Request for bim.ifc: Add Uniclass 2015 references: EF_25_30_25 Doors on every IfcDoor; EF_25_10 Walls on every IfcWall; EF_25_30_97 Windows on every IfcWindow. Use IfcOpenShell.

First a look at what the model holds.

```python
import ifcopenshell

model = ifcopenshell.open("bim.ifc")
print(model.schema)
print("classifications:", [c.Name for c in model.by_type("IfcClassification")])
for ifc_class in ("IfcDoor", "IfcRoof", "IfcStair", "IfcWall", "IfcWindow"):
    print(ifc_class, len(model.by_type(ifc_class)))
```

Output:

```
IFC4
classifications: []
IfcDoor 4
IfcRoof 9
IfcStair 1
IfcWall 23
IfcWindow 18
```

```python
import ifcopenshell
import ifcopenshell.api.classification

model = ifcopenshell.open("bim.ifc")

system = ifcopenshell.api.classification.add_classification(model, classification="Uniclass 2015")

codes = {
    "IfcDoor": ("EF_25_30_25", "Doors"),
    "IfcWall": ("EF_25_10", "Walls"),
    "IfcWindow": ("EF_25_30_97", "Windows"),
}
for ifc_class, (code, name) in codes.items():
    products = model.by_type(ifc_class)
    ifcopenshell.api.classification.add_reference(
        model, products=products, classification=system, identification=code, name=name
    )
    print(code, len(products))

model.write("bim_updated.ifc")
```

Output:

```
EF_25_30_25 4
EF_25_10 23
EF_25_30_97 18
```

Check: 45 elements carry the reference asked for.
